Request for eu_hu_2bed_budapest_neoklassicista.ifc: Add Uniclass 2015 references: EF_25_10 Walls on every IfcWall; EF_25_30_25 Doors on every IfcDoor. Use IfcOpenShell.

First a look at what the model holds.

```python
import ifcopenshell

model = ifcopenshell.open("eu_hu_2bed_budapest_neoklassicista.ifc")
print(model.schema)
print("classifications:", [c.Name for c in model.by_type("IfcClassification")])
for ifc_class in ("IfcDoor", "IfcRoof", "IfcStair", "IfcWall", "IfcWindow"):
    print(ifc_class, len(model.by_type(ifc_class)))
```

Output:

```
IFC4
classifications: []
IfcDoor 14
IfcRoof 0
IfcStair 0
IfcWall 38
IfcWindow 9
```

```python
import ifcopenshell
import ifcopenshell.api.classification

model = ifcopenshell.open("eu_hu_2bed_budapest_neoklassicista.ifc")

system = ifcopenshell.api.classification.add_classification(model, classification="Uniclass 2015")

codes = {
    "IfcWall": ("EF_25_10", "Walls"),
    "IfcDoor": ("EF_25_30_25", "Doors"),
}
for ifc_class, (code, name) in codes.items():
    products = model.by_type(ifc_class)
    ifcopenshell.api.classification.add_reference(
        model, products=products, classification=system, identification=code, name=name
    )
    print(code, len(products))

model.write("eu_hu_2bed_budapest_neoklassicista_rev.ifc")
```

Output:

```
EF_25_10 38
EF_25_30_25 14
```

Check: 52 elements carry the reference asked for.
